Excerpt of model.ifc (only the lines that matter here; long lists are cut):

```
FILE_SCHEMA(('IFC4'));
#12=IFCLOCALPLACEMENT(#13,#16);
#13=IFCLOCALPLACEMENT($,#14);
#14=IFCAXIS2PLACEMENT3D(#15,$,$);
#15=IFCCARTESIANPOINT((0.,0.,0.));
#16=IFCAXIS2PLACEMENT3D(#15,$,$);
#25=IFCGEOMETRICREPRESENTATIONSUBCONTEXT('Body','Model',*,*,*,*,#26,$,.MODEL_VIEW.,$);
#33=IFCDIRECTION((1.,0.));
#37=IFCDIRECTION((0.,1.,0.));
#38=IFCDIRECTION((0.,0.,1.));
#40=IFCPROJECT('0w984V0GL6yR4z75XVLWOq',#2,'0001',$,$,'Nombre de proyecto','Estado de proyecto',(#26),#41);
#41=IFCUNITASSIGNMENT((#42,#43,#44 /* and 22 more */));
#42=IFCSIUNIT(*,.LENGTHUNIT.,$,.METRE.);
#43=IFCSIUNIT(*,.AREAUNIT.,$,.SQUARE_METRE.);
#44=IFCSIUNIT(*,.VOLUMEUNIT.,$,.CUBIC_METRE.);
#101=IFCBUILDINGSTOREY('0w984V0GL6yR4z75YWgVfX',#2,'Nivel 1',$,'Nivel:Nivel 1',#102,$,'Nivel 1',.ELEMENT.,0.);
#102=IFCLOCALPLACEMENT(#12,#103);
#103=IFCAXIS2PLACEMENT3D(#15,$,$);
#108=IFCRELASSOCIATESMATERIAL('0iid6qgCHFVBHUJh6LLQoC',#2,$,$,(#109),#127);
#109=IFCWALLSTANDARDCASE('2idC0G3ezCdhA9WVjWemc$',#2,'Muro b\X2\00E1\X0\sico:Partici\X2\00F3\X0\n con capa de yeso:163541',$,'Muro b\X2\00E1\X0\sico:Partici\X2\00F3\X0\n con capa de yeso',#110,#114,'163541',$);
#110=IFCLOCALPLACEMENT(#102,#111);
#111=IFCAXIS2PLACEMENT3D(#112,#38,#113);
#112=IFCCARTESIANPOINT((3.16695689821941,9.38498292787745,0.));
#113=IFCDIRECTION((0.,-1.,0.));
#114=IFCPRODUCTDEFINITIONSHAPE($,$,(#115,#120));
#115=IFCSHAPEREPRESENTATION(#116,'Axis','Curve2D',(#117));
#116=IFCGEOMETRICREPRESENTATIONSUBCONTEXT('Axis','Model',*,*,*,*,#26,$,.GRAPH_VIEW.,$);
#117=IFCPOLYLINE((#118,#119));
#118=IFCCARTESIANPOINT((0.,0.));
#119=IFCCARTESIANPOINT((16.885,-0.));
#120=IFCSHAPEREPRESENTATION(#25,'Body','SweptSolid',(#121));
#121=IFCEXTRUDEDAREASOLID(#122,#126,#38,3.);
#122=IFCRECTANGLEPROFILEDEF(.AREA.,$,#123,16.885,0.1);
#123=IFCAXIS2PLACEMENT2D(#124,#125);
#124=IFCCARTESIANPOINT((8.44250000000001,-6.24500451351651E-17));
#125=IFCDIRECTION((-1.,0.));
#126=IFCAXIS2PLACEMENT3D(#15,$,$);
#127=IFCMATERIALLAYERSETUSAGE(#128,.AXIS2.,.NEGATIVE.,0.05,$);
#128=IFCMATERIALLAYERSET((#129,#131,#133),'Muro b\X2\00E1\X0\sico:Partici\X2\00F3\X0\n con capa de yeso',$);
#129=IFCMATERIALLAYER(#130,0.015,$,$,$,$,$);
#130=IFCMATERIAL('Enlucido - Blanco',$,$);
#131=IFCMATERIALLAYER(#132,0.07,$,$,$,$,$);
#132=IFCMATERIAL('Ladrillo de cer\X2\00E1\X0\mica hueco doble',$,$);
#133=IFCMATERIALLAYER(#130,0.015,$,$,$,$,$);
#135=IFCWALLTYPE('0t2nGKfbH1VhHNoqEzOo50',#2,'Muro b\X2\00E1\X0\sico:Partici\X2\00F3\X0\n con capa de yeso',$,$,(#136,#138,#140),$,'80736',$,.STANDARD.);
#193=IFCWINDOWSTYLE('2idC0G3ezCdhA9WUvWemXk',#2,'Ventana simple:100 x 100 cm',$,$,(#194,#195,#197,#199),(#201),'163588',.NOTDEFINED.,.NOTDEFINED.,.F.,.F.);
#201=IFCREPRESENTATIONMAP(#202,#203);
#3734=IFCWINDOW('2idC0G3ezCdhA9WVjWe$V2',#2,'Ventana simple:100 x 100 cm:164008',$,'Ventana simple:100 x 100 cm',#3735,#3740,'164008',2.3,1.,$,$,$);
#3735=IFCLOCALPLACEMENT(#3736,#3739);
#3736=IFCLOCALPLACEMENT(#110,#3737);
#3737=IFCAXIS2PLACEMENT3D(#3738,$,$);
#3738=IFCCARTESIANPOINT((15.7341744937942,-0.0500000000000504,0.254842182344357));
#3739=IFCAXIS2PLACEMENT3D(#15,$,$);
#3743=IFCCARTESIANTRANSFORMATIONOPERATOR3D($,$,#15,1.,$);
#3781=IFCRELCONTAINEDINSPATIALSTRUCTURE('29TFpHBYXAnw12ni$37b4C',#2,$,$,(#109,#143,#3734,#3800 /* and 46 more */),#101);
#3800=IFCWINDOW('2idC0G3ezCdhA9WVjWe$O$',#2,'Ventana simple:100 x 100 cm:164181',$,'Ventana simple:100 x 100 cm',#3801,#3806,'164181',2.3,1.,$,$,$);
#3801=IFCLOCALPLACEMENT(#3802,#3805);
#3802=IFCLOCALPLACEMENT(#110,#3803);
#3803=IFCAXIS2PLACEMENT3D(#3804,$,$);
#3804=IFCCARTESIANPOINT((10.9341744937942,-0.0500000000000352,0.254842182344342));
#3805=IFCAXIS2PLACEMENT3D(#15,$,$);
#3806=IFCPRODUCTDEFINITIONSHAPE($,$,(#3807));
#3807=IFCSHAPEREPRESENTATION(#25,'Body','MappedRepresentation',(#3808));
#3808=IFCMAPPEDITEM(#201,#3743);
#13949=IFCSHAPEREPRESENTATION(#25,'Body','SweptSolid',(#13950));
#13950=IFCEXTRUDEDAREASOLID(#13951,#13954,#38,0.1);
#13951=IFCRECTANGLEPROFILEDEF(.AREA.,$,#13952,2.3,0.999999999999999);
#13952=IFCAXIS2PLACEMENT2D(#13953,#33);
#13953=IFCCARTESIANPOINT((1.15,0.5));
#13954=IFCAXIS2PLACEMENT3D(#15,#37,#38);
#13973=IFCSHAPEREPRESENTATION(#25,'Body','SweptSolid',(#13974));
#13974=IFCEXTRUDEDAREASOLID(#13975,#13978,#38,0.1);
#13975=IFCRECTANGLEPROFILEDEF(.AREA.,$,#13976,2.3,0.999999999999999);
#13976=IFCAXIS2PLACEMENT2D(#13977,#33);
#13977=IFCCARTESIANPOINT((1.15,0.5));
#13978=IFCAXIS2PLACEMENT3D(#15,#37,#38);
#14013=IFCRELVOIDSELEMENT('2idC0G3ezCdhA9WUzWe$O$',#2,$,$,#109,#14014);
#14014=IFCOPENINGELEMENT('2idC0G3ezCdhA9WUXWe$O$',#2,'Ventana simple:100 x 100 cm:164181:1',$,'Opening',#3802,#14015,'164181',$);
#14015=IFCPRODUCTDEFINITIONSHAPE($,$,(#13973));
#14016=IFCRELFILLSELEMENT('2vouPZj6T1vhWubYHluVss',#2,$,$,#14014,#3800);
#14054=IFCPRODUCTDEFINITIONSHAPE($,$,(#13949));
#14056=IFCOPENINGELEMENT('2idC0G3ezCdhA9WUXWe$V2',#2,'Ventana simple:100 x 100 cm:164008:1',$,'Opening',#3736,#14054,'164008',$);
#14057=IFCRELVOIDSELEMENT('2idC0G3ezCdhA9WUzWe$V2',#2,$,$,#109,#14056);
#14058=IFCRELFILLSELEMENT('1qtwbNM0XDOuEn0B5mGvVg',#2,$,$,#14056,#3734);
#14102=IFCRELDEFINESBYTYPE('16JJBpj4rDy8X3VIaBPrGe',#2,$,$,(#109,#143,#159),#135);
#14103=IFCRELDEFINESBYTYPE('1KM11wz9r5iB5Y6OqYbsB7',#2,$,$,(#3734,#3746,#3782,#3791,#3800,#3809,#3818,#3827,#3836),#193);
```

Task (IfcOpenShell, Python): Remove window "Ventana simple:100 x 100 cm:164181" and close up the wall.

```python
import ifcopenshell
import ifcopenshell.api.feature
import ifcopenshell.api.root
import ifcopenshell.geom
import ifcopenshell.util.shape

model = ifcopenshell.open("model.ifc")
settings = ifcopenshell.geom.settings()


def volume(element):
    """Net volume in cubic metres, openings subtracted."""
    shape = ifcopenshell.geom.create_shape(settings, element)
    return ifcopenshell.util.shape.get_volume(shape.geometry)


window = model.by_id(3800)
opening = window.FillsVoids[0].RelatingOpeningElement
wall = opening.VoidsElements[0].RelatingBuildingElement
before = volume(wall)

ifcopenshell.api.root.remove_product(model, product=window)
ifcopenshell.api.feature.remove_feature(model, feature=opening)

after = volume(wall)

print(f"wall volume {before:.3f} -> {after:.3f} m3")

model.write("model_rev.ifc")
```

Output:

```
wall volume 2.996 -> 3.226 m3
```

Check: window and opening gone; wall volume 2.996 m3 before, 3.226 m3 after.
